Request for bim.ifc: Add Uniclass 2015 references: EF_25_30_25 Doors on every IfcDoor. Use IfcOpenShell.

First a look at what the model holds.

```python
import ifcopenshell

model = ifcopenshell.open("bim.ifc")
print(model.schema)
print("classifications:", [c.Name for c in model.by_type("IfcClassification")])
for ifc_class in ("IfcDoor", "IfcRoof", "IfcStair", "IfcWall", "IfcWindow"):
    print(ifc_class, len(model.by_type(ifc_class)))
```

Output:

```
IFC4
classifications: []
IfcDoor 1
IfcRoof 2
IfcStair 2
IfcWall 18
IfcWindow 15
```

```python
import ifcopenshell
import ifcopenshell.api.classification

model = ifcopenshell.open("bim.ifc")

system = ifcopenshell.api.classification.add_classification(model, classification="Uniclass 2015")

codes = {
    "IfcDoor": ("EF_25_30_25", "Doors"),
}
for ifc_class, (code, name) in codes.items():
    products = model.by_type(ifc_class)
    ifcopenshell.api.classification.add_reference(
        model, products=products, classification=system, identification=code, name=name
    )
    print(code, len(products))

model.write("bim_updated.ifc")
```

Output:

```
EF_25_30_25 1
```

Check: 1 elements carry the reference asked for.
